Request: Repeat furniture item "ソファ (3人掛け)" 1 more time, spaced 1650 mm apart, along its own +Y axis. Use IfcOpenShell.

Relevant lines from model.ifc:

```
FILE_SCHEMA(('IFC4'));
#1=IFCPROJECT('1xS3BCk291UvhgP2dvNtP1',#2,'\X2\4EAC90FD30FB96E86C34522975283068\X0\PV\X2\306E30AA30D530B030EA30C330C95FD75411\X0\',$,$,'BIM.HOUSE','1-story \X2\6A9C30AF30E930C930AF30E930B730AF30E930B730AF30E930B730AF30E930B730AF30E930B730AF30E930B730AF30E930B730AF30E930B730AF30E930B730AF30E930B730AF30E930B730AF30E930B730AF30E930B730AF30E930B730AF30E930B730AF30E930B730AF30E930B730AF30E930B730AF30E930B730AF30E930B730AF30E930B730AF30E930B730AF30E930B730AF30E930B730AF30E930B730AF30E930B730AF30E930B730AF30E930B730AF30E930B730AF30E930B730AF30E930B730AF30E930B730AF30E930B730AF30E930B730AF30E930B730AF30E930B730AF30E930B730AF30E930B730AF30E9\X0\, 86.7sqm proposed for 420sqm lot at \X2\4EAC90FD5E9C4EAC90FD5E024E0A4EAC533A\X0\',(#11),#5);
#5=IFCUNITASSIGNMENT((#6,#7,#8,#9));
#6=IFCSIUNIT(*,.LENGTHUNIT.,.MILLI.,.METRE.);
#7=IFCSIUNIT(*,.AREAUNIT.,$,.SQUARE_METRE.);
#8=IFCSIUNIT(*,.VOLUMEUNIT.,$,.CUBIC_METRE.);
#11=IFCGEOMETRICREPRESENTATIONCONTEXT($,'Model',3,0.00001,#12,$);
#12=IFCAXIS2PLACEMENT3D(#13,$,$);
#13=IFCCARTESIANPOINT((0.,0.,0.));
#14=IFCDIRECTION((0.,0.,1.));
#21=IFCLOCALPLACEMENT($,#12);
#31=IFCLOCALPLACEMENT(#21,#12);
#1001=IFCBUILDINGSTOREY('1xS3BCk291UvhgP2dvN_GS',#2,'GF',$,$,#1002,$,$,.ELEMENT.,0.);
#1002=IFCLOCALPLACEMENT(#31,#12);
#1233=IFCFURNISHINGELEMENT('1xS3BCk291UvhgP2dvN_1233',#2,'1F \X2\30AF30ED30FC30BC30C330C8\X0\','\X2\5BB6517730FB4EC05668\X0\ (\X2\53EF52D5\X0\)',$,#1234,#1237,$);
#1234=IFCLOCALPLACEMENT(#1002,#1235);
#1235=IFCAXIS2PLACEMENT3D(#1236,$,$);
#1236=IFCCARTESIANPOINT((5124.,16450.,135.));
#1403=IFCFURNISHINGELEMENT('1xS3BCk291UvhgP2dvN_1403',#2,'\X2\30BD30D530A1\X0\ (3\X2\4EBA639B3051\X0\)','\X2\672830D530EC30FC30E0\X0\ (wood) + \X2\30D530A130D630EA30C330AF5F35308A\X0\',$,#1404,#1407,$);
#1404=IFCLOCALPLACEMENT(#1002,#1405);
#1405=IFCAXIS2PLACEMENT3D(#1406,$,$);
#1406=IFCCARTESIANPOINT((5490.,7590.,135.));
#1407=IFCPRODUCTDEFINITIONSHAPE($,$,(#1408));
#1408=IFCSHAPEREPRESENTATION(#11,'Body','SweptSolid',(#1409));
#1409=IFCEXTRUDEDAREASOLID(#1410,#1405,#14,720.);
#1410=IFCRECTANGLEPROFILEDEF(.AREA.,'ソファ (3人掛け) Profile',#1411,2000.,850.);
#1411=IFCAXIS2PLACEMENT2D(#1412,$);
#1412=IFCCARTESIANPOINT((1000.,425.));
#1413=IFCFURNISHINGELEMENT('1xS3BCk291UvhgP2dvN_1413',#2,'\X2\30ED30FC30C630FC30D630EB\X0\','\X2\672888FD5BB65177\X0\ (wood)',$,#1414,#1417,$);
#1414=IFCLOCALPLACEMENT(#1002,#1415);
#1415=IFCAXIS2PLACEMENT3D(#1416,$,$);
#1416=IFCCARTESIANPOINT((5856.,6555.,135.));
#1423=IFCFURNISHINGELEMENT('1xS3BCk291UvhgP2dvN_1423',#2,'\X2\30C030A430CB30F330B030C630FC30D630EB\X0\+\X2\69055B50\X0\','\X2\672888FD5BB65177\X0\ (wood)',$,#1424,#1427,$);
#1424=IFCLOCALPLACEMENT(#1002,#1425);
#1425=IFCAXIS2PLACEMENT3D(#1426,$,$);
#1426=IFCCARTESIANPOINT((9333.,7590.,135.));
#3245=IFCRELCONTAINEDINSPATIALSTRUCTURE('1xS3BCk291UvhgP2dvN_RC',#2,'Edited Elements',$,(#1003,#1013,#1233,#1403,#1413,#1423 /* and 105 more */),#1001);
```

```python
import ifcopenshell
import ifcopenshell.api.geometry
import ifcopenshell.api.root
import ifcopenshell.util.element
import ifcopenshell.util.placement
import ifcopenshell.util.unit

model = ifcopenshell.open("model.ifc")
unit_scale = ifcopenshell.util.unit.calculate_unit_scale(model)


def reuse_history(source, copy):
    """copy_class also copies each property set's owner history, people and application; keep the originals."""
    for rel in copy.IsDefinedBy:
        if rel.is_a("IfcRelDefinesByProperties") and (history := rel.RelatingPropertyDefinition.OwnerHistory):
            rel.RelatingPropertyDefinition.OwnerHistory = source.OwnerHistory
            ifcopenshell.util.element.remove_deep2(model, history)


source = model.by_id(1403)
base = ifcopenshell.util.placement.get_local_placement(source.ObjectPlacement)
step = base[:3, 1] * 1.65 / unit_scale

for i in range(1, 2):
    copy = ifcopenshell.api.root.copy_class(model, product=source)
    copy.Representation = ifcopenshell.util.element.copy_deep(
        model, source.Representation, exclude=["IfcGeometricRepresentationContext", "IfcRepresentationMap"]
    )
    reuse_history(source, copy)
    matrix = base.copy()
    matrix[:3, 3] += i * step
    print("added at", matrix[:3, 3].round(3) + 0.0)
    ifcopenshell.api.geometry.edit_object_placement(model, product=copy, matrix=matrix, is_si=False)

model.write("model_updated.ifc")
```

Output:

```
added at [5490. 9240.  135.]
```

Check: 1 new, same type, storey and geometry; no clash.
